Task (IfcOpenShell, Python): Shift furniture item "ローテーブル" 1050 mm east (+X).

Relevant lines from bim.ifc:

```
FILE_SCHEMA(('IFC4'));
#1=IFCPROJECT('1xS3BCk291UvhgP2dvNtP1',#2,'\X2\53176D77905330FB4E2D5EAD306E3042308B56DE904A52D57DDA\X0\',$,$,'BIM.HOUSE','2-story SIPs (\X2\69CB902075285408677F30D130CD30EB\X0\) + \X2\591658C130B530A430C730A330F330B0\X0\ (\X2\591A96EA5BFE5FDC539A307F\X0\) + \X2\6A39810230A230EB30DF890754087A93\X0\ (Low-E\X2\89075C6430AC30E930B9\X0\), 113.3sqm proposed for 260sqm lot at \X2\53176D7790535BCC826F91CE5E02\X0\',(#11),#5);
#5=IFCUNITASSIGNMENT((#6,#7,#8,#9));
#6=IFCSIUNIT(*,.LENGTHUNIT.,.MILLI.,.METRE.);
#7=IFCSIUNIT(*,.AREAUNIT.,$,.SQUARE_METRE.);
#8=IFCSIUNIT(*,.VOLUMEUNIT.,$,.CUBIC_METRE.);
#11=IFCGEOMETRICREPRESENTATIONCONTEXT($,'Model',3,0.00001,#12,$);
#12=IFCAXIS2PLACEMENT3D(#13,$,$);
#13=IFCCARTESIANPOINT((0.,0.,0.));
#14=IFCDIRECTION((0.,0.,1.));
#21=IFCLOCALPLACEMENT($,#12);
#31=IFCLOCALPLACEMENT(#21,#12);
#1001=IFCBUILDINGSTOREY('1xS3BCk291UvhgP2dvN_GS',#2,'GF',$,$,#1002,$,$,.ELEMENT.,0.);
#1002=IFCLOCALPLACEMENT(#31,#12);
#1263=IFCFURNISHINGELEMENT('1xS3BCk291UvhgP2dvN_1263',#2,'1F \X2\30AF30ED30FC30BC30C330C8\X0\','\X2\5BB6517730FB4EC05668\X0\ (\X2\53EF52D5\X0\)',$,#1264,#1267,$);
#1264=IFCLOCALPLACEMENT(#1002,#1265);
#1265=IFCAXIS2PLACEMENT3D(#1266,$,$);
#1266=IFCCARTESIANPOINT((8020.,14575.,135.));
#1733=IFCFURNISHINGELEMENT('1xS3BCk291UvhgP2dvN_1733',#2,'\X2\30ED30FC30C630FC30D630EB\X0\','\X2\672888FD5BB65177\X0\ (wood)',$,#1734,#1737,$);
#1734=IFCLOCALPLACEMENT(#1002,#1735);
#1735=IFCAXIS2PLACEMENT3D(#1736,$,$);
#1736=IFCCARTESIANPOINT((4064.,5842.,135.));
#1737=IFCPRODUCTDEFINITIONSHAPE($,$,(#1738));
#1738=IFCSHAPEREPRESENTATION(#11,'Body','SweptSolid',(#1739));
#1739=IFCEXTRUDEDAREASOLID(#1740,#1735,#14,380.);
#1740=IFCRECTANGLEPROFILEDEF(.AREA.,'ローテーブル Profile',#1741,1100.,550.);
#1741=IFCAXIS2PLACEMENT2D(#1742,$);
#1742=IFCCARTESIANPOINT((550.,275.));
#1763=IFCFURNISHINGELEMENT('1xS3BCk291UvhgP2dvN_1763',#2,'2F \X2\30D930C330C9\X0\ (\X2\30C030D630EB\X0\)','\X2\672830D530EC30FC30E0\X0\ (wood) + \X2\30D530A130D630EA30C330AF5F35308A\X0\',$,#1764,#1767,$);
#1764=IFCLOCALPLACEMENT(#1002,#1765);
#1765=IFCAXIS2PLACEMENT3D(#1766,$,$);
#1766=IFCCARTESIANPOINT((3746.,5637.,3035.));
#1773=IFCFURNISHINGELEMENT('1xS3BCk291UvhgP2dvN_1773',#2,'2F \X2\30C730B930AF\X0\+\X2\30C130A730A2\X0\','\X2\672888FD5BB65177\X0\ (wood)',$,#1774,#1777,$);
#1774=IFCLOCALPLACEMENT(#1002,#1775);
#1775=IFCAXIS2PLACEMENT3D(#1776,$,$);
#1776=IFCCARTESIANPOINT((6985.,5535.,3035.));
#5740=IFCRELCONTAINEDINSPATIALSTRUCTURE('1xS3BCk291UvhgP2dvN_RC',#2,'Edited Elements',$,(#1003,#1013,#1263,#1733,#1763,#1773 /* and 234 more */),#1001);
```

```python
import ifcopenshell
import ifcopenshell.api.geometry
import ifcopenshell.util.placement

model = ifcopenshell.open("bim.ifc")

item = model.by_guid("1xS3BCk291UvhgP2dvN_1733")
matrix = ifcopenshell.util.placement.get_local_placement(item.ObjectPlacement)
matrix[0, 3] += 1050.0
ifcopenshell.api.geometry.edit_object_placement(model, product=item, matrix=matrix, is_si=False)

print(ifcopenshell.util.placement.get_local_placement(item.ObjectPlacement).round(3) + 0.0)

model.write("bim_rev.ifc")
```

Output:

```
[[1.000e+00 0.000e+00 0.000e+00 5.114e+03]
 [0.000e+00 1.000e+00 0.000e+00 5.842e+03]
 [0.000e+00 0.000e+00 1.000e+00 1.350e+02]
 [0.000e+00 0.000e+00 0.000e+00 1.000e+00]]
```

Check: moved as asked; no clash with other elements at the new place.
